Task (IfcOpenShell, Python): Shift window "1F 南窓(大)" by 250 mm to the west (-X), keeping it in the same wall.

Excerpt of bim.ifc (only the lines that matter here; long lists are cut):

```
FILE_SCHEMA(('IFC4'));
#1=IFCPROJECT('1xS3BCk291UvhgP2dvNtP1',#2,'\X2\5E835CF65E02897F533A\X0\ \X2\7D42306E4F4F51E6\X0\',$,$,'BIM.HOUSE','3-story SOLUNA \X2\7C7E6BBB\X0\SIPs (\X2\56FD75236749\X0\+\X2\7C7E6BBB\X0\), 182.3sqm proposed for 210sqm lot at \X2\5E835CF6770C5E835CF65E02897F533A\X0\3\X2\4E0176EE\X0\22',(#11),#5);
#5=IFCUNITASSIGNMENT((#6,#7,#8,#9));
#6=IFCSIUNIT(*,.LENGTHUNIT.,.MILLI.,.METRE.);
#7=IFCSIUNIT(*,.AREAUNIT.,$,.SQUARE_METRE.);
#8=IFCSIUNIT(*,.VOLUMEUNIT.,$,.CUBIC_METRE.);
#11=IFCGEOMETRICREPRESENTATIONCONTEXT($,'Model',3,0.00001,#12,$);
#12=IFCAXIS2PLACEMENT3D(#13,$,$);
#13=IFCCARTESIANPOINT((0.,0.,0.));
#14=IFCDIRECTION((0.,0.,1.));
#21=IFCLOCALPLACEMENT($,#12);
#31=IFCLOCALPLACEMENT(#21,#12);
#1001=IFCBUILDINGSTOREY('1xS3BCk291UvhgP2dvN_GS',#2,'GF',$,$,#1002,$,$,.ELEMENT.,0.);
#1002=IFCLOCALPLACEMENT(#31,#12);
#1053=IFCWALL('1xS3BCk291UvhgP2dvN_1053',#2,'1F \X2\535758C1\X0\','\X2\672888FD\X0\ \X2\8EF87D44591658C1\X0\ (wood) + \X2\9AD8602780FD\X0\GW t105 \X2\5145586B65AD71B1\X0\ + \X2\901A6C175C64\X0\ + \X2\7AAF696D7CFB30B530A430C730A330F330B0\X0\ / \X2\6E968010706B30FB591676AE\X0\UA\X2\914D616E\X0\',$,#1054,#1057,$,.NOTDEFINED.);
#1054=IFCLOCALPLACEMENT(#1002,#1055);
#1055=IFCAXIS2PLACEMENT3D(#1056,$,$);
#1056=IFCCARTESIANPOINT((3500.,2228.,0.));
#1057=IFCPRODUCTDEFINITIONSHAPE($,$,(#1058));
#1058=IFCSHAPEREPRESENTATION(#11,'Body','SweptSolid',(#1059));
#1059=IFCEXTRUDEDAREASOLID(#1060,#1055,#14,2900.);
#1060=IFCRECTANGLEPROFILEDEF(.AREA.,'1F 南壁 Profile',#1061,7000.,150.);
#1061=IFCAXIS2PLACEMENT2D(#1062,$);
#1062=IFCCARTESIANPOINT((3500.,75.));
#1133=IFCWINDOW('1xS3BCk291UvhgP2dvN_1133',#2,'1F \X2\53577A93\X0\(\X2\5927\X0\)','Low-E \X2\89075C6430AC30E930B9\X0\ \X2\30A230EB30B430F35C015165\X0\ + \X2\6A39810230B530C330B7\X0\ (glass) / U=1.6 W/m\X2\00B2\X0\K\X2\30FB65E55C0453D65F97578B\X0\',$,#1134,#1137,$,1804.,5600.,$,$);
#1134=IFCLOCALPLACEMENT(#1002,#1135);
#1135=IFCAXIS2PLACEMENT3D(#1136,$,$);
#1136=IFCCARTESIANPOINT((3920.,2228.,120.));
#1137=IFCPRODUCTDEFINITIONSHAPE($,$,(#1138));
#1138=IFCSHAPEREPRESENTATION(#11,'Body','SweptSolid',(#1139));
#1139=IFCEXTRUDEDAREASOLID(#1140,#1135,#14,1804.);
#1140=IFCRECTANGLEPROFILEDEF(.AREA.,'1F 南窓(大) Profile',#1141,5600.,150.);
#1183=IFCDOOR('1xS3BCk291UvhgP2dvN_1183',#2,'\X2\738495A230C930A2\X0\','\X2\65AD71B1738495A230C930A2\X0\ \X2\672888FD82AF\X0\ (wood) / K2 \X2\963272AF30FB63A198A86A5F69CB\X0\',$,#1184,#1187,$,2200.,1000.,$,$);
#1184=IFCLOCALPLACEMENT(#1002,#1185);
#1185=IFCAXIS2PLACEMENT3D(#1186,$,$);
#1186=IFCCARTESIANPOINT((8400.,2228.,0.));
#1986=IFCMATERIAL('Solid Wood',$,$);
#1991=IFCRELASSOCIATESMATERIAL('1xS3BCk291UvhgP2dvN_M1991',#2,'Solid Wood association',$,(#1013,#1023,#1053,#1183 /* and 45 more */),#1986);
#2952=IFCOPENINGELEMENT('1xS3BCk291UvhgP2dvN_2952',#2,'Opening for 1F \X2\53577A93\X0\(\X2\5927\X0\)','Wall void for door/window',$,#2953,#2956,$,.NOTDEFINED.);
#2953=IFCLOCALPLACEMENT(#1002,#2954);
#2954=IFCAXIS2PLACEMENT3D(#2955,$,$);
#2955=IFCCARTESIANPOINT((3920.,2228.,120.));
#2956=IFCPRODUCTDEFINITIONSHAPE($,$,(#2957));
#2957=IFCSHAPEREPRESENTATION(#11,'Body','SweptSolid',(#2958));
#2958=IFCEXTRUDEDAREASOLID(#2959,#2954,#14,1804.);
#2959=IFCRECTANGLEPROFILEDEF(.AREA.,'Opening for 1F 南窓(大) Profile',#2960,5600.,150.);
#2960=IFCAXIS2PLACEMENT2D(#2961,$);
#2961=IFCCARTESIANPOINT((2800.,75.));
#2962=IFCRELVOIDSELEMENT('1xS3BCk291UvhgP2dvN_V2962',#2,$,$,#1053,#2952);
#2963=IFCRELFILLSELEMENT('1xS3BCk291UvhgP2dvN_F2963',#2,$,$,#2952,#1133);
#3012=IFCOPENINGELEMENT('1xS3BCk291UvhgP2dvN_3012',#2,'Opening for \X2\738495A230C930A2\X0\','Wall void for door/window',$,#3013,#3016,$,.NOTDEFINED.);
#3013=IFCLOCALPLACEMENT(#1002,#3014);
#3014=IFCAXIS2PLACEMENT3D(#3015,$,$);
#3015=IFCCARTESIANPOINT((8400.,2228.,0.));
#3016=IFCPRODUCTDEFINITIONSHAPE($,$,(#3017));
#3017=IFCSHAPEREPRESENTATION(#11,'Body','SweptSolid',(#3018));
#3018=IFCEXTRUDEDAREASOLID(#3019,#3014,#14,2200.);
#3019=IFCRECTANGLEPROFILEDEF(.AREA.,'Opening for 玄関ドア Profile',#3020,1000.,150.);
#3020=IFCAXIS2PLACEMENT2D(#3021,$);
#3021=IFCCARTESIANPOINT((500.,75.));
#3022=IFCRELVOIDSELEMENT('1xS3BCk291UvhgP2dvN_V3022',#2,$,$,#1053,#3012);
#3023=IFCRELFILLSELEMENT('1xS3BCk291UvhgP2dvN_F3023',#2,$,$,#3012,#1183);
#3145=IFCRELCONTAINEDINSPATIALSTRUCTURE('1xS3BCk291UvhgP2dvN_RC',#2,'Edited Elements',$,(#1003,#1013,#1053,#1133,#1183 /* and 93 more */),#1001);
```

```python
import ifcopenshell
import ifcopenshell.api.geometry
import ifcopenshell.util.placement

model = ifcopenshell.open("bim.ifc")

window = model.by_guid("1xS3BCk291UvhgP2dvN_1133")
opening = window.FillsVoids[0].RelatingOpeningElement
wall = opening.VoidsElements[0].RelatingBuildingElement

wall_matrix = ifcopenshell.util.placement.get_local_placement(wall.ObjectPlacement)
shift = wall_matrix[:3, 0] * -250.0
before = ifcopenshell.util.placement.get_local_placement(window.ObjectPlacement)[:3, 3].copy()

# The window is not placed relative to its opening, so move both.
for product in (opening, window):
    matrix = ifcopenshell.util.placement.get_local_placement(product.ObjectPlacement)
    matrix[:3, 3] += shift
    ifcopenshell.api.geometry.edit_object_placement(model, product=product, matrix=matrix, is_si=False)

after = ifcopenshell.util.placement.get_local_placement(window.ObjectPlacement)[:3, 3]
print("window moved by", (after - before).round(3) + 0.0)

model.write("bim_v2.ifc")
```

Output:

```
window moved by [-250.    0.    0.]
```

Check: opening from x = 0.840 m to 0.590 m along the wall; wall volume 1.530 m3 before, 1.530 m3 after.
